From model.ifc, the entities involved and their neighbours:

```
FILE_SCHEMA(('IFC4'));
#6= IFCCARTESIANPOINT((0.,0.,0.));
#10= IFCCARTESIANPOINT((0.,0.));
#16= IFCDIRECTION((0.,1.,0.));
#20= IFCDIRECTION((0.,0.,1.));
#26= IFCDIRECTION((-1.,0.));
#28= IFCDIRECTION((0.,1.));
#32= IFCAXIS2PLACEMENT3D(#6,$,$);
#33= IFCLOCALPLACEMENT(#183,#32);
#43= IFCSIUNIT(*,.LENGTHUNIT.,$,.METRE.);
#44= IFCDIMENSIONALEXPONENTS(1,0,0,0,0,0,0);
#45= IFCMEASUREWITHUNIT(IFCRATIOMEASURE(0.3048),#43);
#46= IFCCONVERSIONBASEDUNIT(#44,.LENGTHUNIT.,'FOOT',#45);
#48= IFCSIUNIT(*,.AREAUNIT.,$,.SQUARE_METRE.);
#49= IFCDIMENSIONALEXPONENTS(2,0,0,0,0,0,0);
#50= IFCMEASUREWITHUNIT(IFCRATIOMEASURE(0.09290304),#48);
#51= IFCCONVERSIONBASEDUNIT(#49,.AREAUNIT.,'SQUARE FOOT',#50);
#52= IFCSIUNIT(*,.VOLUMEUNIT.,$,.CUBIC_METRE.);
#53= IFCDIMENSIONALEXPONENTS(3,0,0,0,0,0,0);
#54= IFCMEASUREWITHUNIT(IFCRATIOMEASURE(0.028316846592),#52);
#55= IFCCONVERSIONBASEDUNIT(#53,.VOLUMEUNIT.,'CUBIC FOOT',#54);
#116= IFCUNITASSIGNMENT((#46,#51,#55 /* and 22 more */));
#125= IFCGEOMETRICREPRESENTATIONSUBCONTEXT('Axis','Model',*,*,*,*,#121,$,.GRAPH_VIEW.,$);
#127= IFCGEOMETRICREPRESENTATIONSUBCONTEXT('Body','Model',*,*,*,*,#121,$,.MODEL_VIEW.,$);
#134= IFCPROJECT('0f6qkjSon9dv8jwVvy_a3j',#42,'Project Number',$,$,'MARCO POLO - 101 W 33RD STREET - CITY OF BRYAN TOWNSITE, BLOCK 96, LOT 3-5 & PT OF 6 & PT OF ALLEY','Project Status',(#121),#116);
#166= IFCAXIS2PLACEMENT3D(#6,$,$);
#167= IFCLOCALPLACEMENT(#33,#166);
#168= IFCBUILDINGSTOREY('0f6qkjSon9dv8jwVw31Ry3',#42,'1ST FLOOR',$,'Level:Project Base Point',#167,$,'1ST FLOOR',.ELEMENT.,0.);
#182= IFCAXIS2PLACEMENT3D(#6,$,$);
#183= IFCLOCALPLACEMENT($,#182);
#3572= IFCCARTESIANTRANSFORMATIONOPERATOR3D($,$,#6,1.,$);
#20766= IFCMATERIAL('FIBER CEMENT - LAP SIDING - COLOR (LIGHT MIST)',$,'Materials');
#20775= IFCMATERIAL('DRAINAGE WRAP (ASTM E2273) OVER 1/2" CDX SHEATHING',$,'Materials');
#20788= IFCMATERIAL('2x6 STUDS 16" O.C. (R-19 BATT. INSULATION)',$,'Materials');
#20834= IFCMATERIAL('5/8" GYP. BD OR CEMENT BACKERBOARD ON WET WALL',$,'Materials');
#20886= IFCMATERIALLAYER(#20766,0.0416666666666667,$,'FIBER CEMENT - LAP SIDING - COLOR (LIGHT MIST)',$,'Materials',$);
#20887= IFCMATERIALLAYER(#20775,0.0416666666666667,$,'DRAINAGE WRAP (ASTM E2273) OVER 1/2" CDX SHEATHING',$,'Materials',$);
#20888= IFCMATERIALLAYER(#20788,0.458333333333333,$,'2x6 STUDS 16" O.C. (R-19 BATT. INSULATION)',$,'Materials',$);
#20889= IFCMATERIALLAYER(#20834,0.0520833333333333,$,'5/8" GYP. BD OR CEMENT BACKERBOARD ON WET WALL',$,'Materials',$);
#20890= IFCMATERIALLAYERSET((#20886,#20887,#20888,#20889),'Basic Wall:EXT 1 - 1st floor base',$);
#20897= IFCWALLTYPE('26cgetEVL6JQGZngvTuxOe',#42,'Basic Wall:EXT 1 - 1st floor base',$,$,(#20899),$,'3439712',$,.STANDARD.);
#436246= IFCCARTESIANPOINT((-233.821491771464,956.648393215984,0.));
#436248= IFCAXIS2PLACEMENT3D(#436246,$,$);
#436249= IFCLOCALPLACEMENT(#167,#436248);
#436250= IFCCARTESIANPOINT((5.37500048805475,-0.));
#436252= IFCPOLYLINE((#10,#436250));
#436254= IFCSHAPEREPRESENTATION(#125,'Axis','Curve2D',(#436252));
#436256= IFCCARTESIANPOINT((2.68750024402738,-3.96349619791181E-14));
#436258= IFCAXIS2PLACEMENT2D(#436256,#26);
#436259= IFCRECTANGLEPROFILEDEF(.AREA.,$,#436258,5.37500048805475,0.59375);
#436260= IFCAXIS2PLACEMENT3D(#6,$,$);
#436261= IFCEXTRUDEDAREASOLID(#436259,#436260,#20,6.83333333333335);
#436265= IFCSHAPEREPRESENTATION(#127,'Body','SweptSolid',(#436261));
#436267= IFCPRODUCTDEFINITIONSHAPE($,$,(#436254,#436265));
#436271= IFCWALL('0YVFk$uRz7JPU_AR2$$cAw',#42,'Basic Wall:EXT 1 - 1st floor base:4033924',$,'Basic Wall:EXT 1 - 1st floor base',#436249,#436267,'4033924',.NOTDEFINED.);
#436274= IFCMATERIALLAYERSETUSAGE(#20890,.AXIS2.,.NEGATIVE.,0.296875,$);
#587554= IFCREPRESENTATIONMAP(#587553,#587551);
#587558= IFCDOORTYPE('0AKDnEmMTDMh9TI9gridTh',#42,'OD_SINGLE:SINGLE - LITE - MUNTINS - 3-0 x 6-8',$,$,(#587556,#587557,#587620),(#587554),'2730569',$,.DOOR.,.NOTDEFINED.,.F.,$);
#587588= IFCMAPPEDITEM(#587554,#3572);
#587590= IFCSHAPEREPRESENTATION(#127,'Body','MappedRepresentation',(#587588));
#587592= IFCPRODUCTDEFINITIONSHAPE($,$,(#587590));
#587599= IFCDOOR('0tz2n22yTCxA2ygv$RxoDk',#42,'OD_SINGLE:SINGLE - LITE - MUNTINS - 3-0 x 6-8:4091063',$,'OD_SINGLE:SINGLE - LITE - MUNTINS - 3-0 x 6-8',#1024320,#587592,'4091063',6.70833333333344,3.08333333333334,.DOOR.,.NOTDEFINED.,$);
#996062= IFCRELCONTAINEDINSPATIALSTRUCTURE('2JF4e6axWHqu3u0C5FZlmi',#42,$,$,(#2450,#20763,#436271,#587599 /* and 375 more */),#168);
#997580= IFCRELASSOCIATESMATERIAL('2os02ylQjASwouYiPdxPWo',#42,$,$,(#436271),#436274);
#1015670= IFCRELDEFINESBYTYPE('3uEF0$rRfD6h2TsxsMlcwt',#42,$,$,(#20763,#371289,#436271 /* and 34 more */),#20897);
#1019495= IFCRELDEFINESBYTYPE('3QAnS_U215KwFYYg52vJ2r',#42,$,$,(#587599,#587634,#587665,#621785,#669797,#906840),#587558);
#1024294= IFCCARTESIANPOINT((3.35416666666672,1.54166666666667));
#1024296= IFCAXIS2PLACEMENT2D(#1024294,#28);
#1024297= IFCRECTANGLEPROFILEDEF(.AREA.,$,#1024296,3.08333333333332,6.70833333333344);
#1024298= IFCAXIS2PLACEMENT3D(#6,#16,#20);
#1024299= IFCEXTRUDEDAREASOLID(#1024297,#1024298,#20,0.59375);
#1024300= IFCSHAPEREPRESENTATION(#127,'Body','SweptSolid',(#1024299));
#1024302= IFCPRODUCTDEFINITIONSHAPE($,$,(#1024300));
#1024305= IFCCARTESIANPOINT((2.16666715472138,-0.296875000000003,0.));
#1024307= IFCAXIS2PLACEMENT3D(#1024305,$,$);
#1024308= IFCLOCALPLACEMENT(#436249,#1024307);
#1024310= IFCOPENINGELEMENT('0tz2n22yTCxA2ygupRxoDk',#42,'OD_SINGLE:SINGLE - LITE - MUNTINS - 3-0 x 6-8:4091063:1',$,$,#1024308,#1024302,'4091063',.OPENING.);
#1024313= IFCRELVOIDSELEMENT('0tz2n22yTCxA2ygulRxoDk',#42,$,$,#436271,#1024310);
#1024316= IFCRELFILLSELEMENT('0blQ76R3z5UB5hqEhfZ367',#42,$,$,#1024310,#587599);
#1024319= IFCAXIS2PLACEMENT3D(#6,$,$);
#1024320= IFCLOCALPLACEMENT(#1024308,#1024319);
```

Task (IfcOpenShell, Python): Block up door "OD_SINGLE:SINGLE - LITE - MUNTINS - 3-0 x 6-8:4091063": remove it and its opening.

```python
import ifcopenshell
import ifcopenshell.api.feature
import ifcopenshell.api.root
import ifcopenshell.geom
import ifcopenshell.util.shape

model = ifcopenshell.open("model.ifc")
settings = ifcopenshell.geom.settings()


def volume(element):
    """Net volume in cubic metres, openings subtracted."""
    shape = ifcopenshell.geom.create_shape(settings, element)
    return ifcopenshell.util.shape.get_volume(shape.geometry)


door = model.by_guid("0tz2n22yTCxA2ygv$RxoDk")
opening = door.FillsVoids[0].RelatingOpeningElement
wall = opening.VoidsElements[0].RelatingBuildingElement
before = volume(wall)

ifcopenshell.api.root.remove_product(model, product=door)
ifcopenshell.api.feature.remove_feature(model, feature=opening)

after = volume(wall)

print(f"wall volume {before:.3f} -> {after:.3f} m3")

model.write("model_updated.ifc")
```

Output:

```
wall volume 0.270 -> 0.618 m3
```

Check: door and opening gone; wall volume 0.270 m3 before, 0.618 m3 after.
